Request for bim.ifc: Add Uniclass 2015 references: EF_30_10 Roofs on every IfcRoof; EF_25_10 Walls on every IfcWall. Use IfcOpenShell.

First a look at what the model holds.

```python
import ifcopenshell

model = ifcopenshell.open("bim.ifc")
print(model.schema)
print("classifications:", [c.Name for c in model.by_type("IfcClassification")])
for ifc_class in ("IfcDoor", "IfcRoof", "IfcStair", "IfcWall", "IfcWindow"):
    print(ifc_class, len(model.by_type(ifc_class)))
```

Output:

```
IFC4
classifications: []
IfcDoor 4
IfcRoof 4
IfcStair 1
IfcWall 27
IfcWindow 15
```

```python
import ifcopenshell
import ifcopenshell.api.classification

model = ifcopenshell.open("bim.ifc")

system = ifcopenshell.api.classification.add_classification(model, classification="Uniclass 2015")

codes = {
    "IfcRoof": ("EF_30_10", "Roofs"),
    "IfcWall": ("EF_25_10", "Walls"),
}
for ifc_class, (code, name) in codes.items():
    products = model.by_type(ifc_class)
    ifcopenshell.api.classification.add_reference(
        model, products=products, classification=system, identification=code, name=name
    )
    print(code, len(products))

model.write("bim-out.ifc")
```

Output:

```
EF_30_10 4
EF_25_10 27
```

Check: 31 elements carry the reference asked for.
